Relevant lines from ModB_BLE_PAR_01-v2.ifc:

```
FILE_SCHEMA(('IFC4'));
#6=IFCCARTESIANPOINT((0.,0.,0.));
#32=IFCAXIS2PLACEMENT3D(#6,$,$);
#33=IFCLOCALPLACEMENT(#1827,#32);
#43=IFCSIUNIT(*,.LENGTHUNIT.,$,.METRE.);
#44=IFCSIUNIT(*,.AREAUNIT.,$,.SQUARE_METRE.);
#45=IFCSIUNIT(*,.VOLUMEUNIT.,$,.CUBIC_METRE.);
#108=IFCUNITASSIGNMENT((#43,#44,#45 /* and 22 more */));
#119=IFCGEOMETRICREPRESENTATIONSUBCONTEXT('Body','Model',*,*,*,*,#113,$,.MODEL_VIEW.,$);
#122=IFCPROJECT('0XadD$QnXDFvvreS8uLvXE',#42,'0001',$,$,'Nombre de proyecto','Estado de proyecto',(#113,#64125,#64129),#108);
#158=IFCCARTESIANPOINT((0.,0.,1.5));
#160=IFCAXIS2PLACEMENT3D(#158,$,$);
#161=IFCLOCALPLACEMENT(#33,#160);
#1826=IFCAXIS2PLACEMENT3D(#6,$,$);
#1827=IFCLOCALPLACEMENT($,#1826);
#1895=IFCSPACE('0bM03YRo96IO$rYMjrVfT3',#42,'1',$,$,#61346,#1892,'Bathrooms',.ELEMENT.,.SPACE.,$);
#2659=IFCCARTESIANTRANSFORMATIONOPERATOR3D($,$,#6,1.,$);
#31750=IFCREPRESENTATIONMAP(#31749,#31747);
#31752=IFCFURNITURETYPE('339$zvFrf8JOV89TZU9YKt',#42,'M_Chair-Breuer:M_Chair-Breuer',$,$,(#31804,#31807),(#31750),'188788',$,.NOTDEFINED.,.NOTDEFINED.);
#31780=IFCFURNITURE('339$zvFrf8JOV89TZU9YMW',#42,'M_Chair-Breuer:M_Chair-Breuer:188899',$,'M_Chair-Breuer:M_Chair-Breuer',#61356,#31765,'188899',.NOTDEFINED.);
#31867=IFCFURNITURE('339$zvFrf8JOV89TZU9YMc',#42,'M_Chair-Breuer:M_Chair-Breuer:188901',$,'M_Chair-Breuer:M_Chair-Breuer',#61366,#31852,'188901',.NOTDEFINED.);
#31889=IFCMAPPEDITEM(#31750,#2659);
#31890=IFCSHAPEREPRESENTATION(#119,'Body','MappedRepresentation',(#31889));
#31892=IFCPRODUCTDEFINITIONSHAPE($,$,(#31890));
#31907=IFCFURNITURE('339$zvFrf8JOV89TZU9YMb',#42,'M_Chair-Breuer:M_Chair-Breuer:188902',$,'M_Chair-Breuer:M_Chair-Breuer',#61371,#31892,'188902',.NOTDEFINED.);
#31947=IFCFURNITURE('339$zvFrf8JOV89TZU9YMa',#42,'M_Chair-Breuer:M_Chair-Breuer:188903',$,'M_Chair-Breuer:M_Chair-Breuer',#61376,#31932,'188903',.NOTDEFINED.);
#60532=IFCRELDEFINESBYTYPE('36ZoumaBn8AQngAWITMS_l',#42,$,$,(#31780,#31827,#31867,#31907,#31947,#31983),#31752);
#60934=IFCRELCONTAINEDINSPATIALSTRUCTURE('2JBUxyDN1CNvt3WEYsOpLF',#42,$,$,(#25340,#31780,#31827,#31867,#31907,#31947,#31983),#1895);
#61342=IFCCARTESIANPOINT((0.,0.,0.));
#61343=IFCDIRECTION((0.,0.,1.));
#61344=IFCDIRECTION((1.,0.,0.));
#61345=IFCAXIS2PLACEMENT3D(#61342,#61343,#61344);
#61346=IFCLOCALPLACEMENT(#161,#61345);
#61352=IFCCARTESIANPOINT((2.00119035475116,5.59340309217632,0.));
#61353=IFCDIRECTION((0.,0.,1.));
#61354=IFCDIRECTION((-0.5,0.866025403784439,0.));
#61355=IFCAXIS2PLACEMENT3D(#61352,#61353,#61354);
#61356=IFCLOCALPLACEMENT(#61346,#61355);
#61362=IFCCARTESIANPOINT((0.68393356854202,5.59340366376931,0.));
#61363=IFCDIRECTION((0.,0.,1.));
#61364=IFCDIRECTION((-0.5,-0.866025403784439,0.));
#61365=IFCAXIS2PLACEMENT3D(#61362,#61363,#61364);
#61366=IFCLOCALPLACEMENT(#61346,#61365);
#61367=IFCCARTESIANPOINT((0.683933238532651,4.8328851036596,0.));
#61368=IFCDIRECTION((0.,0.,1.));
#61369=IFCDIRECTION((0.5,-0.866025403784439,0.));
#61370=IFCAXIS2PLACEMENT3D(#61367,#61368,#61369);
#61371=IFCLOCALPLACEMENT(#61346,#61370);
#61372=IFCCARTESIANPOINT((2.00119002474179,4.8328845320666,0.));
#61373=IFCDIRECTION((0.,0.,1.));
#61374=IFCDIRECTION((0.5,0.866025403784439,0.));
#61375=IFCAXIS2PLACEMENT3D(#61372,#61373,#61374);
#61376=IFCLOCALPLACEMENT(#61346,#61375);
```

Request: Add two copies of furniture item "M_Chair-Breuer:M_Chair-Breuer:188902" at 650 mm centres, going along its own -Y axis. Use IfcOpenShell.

```python
import ifcopenshell
import ifcopenshell.api.geometry
import ifcopenshell.api.root
import ifcopenshell.util.element
import ifcopenshell.util.placement
import ifcopenshell.util.unit

model = ifcopenshell.open("ModB_BLE_PAR_01-v2.ifc")
unit_scale = ifcopenshell.util.unit.calculate_unit_scale(model)


def reuse_history(source, copy):
    """copy_class also copies each property set's owner history, people and application; keep the originals."""
    for rel in copy.IsDefinedBy:
        if rel.is_a("IfcRelDefinesByProperties") and (history := rel.RelatingPropertyDefinition.OwnerHistory):
            rel.RelatingPropertyDefinition.OwnerHistory = source.OwnerHistory
            ifcopenshell.util.element.remove_deep2(model, history)


source = model.by_guid("339$zvFrf8JOV89TZU9YMb")
base = ifcopenshell.util.placement.get_local_placement(source.ObjectPlacement)
step = -base[:3, 1] * 0.65 / unit_scale

for i in range(1, 3):
    copy = ifcopenshell.api.root.copy_class(model, product=source)
    copy.Representation = ifcopenshell.util.element.copy_deep(
        model, source.Representation, exclude=["IfcGeometricRepresentationContext", "IfcRepresentationMap"]
    )
    copy.Name = "M_Chair-Breuer:M_Chair-Breuer"
    copy.Tag = None
    reuse_history(source, copy)
    matrix = base.copy()
    matrix[:3, 3] += i * step
    print("added at", matrix[:3, 3].round(3) + 0.0)
    ifcopenshell.api.geometry.edit_object_placement(model, product=copy, matrix=matrix, is_si=False)

model.write("ModB_BLE_PAR_01-v2_updated.ifc")
```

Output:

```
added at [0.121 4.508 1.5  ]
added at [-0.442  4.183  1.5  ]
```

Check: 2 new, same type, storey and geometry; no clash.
